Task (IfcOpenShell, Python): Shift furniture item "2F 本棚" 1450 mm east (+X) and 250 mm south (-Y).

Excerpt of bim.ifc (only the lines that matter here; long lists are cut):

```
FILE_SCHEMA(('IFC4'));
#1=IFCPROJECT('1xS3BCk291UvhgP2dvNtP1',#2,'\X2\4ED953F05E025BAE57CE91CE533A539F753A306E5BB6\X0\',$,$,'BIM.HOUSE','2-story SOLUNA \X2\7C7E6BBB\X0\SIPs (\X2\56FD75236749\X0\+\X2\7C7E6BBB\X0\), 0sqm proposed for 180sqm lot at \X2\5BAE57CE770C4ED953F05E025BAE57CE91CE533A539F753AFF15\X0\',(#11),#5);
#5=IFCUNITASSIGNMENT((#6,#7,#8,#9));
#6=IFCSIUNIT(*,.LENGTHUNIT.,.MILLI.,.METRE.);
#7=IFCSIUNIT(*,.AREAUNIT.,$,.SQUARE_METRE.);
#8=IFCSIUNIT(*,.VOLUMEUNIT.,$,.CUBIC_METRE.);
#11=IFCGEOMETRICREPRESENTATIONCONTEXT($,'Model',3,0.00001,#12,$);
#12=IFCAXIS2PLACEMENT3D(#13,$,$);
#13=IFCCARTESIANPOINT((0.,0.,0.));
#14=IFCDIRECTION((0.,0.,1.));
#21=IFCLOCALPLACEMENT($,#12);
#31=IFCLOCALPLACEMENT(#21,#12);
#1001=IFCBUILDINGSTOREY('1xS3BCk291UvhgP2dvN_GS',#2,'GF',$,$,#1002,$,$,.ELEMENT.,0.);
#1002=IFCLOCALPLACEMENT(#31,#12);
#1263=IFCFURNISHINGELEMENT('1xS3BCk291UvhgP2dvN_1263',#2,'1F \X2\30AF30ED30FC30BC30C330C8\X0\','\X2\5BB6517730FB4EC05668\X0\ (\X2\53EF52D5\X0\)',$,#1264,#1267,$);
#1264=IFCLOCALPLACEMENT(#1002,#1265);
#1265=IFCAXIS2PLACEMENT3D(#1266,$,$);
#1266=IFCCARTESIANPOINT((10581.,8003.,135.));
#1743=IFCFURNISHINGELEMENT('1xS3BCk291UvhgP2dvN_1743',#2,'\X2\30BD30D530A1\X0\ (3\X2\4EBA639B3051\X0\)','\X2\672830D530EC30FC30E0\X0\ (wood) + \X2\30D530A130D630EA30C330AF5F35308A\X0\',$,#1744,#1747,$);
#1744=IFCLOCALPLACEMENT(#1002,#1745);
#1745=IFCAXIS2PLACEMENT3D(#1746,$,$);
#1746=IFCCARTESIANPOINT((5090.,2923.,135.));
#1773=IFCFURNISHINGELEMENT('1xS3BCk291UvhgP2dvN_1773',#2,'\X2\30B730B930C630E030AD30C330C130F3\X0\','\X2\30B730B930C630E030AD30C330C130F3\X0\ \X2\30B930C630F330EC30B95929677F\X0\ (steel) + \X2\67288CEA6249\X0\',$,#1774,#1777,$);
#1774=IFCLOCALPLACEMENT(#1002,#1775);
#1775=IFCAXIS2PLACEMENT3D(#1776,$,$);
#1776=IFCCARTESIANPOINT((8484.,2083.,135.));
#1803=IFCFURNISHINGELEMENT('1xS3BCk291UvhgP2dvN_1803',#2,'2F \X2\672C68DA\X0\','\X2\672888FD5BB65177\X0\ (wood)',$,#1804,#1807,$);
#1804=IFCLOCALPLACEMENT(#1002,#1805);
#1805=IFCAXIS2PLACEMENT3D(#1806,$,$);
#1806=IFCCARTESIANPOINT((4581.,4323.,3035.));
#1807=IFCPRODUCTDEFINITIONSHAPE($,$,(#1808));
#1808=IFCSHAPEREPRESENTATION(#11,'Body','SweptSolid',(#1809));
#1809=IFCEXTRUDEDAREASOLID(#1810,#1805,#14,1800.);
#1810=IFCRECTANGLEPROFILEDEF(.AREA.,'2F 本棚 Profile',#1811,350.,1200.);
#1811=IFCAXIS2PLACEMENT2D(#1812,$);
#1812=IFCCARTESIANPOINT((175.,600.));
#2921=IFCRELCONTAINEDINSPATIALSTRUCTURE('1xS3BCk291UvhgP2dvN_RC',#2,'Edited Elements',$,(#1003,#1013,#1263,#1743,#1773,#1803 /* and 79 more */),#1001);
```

```python
import ifcopenshell
import ifcopenshell.api.geometry
import ifcopenshell.util.placement
import ifcopenshell.util.unit

model = ifcopenshell.open("bim.ifc")
unit_scale = ifcopenshell.util.unit.calculate_unit_scale(model)

item = model.by_guid("1xS3BCk291UvhgP2dvN_1803")
matrix = ifcopenshell.util.placement.get_local_placement(item.ObjectPlacement)
matrix[0, 3] += 1.45 / unit_scale
matrix[1, 3] -= 0.25 / unit_scale
ifcopenshell.api.geometry.edit_object_placement(model, product=item, matrix=matrix, is_si=False)

print(ifcopenshell.util.placement.get_local_placement(item.ObjectPlacement).round(3) + 0.0)

model.write("bim-out.ifc")
```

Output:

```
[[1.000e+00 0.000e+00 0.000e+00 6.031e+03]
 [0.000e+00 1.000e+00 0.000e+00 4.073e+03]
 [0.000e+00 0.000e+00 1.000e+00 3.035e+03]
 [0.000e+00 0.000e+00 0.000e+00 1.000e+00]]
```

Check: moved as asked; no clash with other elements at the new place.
